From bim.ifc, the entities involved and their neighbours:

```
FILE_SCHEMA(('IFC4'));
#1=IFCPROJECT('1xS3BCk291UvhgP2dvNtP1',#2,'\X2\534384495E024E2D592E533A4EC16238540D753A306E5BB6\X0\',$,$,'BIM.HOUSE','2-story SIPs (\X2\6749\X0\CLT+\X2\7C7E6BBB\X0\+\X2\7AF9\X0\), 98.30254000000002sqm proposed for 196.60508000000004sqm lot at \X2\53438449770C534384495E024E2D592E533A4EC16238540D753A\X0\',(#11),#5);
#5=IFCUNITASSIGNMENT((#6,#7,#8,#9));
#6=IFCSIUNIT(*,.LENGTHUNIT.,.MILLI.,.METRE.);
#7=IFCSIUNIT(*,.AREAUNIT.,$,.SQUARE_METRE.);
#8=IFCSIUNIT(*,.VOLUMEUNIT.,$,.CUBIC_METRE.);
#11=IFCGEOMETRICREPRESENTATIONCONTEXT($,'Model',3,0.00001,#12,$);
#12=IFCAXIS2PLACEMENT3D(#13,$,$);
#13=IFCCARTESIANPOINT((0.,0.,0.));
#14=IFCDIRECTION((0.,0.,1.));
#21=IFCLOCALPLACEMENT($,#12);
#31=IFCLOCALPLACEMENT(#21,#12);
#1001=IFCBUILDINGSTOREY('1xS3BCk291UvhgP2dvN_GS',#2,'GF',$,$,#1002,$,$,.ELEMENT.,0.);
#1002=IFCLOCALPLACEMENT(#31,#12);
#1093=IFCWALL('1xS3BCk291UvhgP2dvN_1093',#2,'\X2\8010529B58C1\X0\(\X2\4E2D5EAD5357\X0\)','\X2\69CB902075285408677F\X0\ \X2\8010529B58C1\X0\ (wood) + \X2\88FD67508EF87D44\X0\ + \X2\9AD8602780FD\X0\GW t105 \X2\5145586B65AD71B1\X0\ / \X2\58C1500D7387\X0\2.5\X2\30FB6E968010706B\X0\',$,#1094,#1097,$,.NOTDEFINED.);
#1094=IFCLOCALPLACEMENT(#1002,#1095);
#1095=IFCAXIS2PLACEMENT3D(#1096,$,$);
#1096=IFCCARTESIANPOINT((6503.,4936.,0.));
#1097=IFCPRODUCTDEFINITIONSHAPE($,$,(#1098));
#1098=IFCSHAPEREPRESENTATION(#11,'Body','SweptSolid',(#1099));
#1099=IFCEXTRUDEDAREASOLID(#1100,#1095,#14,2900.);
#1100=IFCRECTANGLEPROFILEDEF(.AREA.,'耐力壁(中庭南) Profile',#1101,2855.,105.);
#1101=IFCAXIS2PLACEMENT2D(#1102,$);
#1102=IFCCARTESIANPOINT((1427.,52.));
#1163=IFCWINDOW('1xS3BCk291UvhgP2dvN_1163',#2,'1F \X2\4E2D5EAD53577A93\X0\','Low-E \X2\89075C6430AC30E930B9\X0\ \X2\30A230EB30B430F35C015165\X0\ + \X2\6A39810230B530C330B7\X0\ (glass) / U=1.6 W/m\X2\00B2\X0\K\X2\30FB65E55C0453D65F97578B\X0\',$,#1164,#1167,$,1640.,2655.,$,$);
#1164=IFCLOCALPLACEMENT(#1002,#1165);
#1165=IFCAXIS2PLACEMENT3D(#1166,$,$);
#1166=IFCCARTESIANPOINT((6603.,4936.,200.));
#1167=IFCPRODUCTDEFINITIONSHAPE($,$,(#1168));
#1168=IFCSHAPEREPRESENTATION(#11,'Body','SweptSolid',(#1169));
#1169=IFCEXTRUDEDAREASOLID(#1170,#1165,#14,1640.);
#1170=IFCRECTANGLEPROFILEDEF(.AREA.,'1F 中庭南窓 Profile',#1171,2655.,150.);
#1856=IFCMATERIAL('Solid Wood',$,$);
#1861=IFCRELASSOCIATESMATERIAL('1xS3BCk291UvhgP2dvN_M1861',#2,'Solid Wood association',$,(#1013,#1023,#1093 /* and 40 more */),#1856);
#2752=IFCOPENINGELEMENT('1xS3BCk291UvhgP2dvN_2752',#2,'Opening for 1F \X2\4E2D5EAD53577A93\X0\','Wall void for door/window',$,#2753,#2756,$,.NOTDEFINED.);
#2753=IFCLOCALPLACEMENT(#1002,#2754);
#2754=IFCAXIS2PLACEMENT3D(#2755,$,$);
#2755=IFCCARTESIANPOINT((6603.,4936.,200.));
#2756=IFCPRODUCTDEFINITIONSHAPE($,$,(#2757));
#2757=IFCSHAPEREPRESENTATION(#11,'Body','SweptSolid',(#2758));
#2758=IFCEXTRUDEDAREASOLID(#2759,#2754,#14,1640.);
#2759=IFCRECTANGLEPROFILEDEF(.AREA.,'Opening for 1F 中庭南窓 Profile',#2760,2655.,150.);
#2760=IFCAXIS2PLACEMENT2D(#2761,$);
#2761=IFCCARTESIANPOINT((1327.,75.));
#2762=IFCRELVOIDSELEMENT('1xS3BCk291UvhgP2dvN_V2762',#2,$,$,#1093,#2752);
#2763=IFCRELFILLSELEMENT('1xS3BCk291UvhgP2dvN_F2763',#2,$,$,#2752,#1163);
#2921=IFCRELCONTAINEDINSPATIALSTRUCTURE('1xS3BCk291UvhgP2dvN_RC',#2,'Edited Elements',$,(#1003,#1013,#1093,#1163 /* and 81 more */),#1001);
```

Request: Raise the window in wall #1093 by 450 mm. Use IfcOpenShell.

```python
import numpy as np
import ifcopenshell
import ifcopenshell.api.geometry
import ifcopenshell.util.placement
import ifcopenshell.util.unit

model = ifcopenshell.open("bim.ifc")
unit_scale = ifcopenshell.util.unit.calculate_unit_scale(model)

window = model.by_id(1163)
opening = window.FillsVoids[0].RelatingOpeningElement
dz = 450.0

shift = np.array([0.0, 0.0, dz])
# The window is not placed relative to its opening, so move both.
for product in (opening, window):
    matrix = ifcopenshell.util.placement.get_local_placement(product.ObjectPlacement)
    matrix[:3, 3] += shift
    ifcopenshell.api.geometry.edit_object_placement(model, product=product, matrix=matrix, is_si=False)

print(f"moved by {dz * unit_scale:+.3f} m")

model.write("bim_v2.ifc")
```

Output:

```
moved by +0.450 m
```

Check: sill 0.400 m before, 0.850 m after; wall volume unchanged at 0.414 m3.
